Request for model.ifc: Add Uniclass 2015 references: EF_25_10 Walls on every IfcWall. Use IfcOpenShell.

First a look at what the model holds.

```python
import ifcopenshell

model = ifcopenshell.open("model.ifc")
print(model.schema)
print("classifications:", [c.Name for c in model.by_type("IfcClassification")])
for ifc_class in ("IfcDoor", "IfcRoof", "IfcStair", "IfcWall", "IfcWindow"):
    print(ifc_class, len(model.by_type(ifc_class)))
```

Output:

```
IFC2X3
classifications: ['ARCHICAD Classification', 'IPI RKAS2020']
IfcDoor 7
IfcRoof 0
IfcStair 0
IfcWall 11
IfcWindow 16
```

```python
import ifcopenshell
import ifcopenshell.api.classification

model = ifcopenshell.open("model.ifc")

# IFC2X3 requires Source and Edition and has no link from the project to the system.
system = model.create_entity("IfcClassification", Source="NBS", Edition="2015", Name="Uniclass 2015")

codes = {
    "IfcWall": ("EF_25_10", "Walls"),
}
for ifc_class, (code, name) in codes.items():
    products = model.by_type(ifc_class)
    ifcopenshell.api.classification.add_reference(
        model, products=products, classification=system, identification=code, name=name
    )
    print(code, len(products))

model.write("model_v2.ifc")
```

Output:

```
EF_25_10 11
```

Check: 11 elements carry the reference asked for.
